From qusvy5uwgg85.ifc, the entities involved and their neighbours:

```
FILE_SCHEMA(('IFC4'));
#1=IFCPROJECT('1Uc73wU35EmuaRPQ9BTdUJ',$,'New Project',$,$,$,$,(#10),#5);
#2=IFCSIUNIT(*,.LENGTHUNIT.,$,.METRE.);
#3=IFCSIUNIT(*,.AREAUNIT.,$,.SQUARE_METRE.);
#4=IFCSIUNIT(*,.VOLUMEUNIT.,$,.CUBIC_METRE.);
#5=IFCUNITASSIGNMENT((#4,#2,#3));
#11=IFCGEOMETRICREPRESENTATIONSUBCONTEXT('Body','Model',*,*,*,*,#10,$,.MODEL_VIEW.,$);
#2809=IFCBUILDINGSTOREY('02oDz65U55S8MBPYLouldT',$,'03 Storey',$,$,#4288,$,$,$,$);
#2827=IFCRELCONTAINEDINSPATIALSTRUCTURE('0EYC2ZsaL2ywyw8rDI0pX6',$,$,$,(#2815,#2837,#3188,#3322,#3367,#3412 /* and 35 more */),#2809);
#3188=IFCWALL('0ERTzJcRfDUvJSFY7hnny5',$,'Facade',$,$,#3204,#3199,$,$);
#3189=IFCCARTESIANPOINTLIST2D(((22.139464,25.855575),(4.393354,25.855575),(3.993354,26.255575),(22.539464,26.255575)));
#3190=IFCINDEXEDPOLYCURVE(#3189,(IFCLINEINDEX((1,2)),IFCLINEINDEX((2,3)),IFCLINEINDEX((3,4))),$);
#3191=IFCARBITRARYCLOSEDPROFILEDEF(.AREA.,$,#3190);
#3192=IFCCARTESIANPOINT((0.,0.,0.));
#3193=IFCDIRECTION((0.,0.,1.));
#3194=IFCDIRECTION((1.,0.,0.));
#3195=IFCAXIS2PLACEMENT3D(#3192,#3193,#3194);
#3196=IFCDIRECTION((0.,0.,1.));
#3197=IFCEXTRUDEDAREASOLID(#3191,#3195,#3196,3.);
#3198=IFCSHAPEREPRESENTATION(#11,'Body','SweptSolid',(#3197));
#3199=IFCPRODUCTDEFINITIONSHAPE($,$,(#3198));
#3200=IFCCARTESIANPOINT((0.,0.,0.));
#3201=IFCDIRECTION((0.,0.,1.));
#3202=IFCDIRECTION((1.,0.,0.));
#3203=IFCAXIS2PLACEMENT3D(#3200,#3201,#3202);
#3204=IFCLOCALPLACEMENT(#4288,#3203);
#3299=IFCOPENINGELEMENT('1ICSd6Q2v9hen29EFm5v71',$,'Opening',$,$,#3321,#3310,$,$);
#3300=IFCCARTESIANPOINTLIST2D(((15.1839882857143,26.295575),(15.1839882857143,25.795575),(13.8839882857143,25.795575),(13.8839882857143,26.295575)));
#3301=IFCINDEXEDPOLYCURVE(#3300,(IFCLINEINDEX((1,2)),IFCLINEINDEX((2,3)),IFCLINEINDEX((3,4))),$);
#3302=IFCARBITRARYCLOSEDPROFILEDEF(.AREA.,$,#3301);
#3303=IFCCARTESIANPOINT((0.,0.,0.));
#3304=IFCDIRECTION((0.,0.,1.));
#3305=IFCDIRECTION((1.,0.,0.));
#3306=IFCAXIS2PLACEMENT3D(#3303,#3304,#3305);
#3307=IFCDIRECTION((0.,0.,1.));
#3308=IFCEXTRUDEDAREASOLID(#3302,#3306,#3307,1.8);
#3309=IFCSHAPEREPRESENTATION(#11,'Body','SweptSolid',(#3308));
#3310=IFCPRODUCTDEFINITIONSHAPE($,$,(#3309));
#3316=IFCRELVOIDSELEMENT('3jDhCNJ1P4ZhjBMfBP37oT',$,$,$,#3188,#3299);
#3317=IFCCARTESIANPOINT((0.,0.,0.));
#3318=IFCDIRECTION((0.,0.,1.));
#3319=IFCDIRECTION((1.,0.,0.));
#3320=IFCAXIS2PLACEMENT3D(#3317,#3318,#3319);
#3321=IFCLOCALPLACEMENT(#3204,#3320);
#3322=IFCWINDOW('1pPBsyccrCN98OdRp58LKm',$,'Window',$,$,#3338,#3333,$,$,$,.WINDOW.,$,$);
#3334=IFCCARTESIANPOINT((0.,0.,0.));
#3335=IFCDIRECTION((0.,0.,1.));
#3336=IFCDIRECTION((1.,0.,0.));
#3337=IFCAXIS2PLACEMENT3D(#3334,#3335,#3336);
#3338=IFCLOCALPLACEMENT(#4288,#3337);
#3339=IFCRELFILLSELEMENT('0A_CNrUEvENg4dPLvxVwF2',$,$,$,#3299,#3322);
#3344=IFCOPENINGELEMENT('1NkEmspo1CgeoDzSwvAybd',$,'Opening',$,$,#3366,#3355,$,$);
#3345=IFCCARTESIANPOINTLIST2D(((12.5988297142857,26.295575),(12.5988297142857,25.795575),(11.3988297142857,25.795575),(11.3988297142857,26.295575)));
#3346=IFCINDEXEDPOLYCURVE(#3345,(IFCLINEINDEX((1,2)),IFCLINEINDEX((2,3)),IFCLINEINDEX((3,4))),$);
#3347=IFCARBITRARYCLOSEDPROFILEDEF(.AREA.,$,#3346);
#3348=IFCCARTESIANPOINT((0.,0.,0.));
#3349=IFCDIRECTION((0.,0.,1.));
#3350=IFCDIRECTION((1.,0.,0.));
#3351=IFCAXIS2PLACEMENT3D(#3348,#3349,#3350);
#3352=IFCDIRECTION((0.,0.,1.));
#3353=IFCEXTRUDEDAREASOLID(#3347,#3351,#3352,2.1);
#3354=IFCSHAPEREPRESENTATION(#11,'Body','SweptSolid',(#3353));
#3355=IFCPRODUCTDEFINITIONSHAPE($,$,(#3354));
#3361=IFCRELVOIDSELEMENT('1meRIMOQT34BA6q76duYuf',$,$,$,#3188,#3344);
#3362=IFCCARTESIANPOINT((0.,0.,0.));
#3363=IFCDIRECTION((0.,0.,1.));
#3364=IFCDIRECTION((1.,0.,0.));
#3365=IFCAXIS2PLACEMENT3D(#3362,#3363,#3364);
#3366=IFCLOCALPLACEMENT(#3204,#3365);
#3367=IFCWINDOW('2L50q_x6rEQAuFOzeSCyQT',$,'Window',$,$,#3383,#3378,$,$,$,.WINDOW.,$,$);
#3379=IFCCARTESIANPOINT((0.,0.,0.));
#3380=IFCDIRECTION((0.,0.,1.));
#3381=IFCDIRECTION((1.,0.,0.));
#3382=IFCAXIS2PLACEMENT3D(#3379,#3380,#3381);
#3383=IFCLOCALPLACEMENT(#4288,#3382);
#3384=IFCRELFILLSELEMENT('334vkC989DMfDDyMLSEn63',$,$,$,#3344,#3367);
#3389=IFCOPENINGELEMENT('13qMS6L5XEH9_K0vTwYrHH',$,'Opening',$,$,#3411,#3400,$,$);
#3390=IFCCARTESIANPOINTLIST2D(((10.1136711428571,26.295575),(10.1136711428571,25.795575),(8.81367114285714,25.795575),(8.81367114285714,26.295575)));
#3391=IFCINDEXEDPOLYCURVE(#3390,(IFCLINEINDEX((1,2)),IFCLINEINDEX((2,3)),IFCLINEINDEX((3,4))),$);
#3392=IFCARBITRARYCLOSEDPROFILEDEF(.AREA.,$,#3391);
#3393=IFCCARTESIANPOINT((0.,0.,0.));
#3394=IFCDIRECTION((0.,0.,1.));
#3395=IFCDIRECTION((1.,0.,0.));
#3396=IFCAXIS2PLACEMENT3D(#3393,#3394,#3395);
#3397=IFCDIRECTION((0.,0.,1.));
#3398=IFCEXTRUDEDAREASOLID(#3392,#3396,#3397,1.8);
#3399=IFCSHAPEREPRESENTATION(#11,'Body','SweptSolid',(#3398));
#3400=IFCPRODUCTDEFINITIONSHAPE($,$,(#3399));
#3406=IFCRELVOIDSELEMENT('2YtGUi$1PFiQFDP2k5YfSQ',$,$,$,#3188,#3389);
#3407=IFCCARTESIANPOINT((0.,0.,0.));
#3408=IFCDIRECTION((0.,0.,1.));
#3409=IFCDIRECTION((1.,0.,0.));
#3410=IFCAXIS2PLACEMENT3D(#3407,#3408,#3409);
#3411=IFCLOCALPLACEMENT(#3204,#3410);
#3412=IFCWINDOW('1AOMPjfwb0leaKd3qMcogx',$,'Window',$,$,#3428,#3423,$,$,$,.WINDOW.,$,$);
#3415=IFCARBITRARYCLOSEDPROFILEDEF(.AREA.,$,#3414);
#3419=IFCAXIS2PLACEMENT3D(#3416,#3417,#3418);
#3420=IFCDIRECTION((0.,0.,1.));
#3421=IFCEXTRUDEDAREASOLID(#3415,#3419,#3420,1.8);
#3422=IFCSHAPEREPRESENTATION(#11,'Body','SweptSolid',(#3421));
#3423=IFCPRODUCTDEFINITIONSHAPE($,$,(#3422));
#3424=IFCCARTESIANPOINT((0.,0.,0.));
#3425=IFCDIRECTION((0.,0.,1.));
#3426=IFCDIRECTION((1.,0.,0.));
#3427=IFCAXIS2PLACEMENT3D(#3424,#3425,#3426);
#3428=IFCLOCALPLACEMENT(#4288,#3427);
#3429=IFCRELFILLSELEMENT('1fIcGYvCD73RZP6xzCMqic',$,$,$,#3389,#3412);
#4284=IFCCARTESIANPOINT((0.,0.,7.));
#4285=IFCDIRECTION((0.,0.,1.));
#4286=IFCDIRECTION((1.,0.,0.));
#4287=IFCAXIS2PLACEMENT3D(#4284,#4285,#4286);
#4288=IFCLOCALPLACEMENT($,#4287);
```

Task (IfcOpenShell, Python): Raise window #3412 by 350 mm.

```python
import numpy as np
import ifcopenshell
import ifcopenshell.api.geometry
import ifcopenshell.util.placement
import ifcopenshell.util.unit

model = ifcopenshell.open("qusvy5uwgg85.ifc")
unit_scale = ifcopenshell.util.unit.calculate_unit_scale(model)

window = model.by_guid("1AOMPjfwb0leaKd3qMcogx")
opening = window.FillsVoids[0].RelatingOpeningElement
dz = 0.35

shift = np.array([0.0, 0.0, dz])
# The window is not placed relative to its opening, so move both.
for product in (opening, window):
    matrix = ifcopenshell.util.placement.get_local_placement(product.ObjectPlacement)
    matrix[:3, 3] += shift
    ifcopenshell.api.geometry.edit_object_placement(model, product=product, matrix=matrix, is_si=False)

print(f"moved by {dz * unit_scale:+.3f} m")

model.write("qusvy5uwgg85_edited.ifc")
```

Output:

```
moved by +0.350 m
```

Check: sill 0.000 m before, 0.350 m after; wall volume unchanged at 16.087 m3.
